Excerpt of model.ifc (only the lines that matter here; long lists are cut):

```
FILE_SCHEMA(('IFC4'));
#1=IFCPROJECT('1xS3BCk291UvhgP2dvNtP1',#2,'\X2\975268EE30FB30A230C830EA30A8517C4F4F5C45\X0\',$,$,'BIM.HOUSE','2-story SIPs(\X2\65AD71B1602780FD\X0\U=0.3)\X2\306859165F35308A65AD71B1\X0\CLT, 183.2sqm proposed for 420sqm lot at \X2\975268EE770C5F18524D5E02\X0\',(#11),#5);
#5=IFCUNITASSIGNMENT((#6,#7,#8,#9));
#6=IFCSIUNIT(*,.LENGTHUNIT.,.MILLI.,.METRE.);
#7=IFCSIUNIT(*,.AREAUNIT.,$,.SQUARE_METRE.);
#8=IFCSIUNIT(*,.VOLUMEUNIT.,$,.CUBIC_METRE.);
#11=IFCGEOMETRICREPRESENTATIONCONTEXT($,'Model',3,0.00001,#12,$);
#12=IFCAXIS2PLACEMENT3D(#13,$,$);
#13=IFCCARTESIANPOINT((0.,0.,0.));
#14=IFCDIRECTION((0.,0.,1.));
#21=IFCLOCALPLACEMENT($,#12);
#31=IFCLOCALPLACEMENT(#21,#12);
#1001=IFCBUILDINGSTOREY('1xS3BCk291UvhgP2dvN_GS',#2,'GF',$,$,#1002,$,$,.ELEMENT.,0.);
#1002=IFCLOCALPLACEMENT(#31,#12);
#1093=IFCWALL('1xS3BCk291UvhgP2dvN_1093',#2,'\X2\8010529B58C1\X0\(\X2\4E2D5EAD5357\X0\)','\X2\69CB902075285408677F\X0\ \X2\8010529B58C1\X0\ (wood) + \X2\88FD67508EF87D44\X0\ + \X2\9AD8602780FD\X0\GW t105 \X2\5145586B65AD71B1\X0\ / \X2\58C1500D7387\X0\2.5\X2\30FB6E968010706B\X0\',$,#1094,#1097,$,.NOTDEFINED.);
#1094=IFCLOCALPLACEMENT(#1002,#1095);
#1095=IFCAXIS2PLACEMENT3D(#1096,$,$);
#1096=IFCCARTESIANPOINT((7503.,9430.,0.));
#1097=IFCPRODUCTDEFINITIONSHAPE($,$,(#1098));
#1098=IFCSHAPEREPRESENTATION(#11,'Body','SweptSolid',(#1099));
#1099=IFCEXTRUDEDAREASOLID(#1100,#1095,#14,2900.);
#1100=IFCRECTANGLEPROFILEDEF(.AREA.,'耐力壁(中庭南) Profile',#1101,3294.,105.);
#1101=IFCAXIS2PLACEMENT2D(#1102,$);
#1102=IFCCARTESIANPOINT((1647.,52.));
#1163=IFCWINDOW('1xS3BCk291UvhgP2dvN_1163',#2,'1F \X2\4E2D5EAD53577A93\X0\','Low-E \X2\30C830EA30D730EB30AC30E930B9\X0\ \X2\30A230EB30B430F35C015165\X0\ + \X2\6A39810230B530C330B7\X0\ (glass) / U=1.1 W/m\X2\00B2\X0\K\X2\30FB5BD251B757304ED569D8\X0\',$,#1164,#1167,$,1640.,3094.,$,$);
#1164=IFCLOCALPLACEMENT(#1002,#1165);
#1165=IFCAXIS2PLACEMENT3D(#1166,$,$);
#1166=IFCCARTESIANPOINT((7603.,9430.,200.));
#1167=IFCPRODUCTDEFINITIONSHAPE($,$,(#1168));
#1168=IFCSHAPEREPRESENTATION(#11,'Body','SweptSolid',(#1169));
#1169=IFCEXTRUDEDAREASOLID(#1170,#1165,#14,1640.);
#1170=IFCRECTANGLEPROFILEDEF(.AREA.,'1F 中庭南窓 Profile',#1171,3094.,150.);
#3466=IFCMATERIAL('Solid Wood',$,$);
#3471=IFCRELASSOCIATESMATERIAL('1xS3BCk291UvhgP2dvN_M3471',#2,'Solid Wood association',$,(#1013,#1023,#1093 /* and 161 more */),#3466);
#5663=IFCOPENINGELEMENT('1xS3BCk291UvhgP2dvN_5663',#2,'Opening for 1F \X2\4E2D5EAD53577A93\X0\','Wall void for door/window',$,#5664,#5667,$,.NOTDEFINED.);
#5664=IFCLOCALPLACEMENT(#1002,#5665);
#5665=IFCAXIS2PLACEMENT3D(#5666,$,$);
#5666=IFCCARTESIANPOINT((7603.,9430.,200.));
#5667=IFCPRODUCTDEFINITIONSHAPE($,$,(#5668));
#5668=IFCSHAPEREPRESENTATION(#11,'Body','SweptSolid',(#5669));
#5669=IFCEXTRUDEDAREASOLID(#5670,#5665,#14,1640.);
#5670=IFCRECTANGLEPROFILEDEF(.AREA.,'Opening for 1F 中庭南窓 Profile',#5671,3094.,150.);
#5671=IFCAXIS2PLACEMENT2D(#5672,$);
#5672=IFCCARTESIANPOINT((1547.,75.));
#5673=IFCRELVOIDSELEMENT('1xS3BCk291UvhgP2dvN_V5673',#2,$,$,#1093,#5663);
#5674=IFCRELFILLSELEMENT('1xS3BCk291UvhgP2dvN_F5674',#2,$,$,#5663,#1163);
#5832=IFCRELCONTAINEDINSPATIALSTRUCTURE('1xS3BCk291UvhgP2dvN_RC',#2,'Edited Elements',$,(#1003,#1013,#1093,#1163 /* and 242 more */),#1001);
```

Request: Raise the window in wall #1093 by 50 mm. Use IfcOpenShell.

```python
import numpy as np
import ifcopenshell
import ifcopenshell.api.geometry
import ifcopenshell.util.placement
import ifcopenshell.util.unit

model = ifcopenshell.open("model.ifc")
unit_scale = ifcopenshell.util.unit.calculate_unit_scale(model)

window = model.by_id(1163)
opening = window.FillsVoids[0].RelatingOpeningElement
dz = 50.0

shift = np.array([0.0, 0.0, dz])
# The window is not placed relative to its opening, so move both.
for product in (opening, window):
    matrix = ifcopenshell.util.placement.get_local_placement(product.ObjectPlacement)
    matrix[:3, 3] += shift
    ifcopenshell.api.geometry.edit_object_placement(model, product=product, matrix=matrix, is_si=False)

print(f"moved by {dz * unit_scale:+.3f} m")

model.write("model_rev.ifc")
```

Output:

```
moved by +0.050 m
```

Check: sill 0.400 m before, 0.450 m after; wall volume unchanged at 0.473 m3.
